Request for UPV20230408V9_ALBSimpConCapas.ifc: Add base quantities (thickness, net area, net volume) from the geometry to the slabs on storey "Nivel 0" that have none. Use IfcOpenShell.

First a look at what the model holds.

```python
import ifcopenshell
import ifcopenshell.util.element
import ifcopenshell.util.unit

model = ifcopenshell.open("UPV20230408V9_ALBSimpConCapas.ifc")
print(model.schema)
for unit_type in ("LENGTHUNIT", "AREAUNIT", "VOLUMEUNIT"):
    print(unit_type, ifcopenshell.util.unit.calculate_unit_scale(model, unit_type))
storey = next(s for s in model.by_type("IfcBuildingStorey") if s.Name == "Nivel 0")
slabs = [e for e in ifcopenshell.util.element.get_decomposition(storey) if e.is_a("IfcSlab")]
for e in sorted(slabs, key=lambda e: e.id()):
    print(e.id(), e.is_a(), e.Name, list(ifcopenshell.util.element.get_psets(e, qtos_only=True)), sep=" | ")
```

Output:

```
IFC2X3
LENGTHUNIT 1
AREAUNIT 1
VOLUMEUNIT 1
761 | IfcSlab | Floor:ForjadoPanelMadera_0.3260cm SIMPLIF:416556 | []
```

```python
import ifcopenshell
import ifcopenshell.api.pset
import ifcopenshell.geom
import ifcopenshell.util.element
import ifcopenshell.util.shape
import ifcopenshell.util.unit

model = ifcopenshell.open("UPV20230408V9_ALBSimpConCapas.ifc")
unit_scale = ifcopenshell.util.unit.calculate_unit_scale(model)
area_scale = ifcopenshell.util.unit.calculate_unit_scale(model, "AREAUNIT")
volume_scale = ifcopenshell.util.unit.calculate_unit_scale(model, "VOLUMEUNIT")
settings = ifcopenshell.geom.settings()

storey = next(s for s in model.by_type("IfcBuildingStorey") if s.Name == "Nivel 0")
slabs = [e for e in ifcopenshell.util.element.get_decomposition(storey) if e.is_a("IfcSlab")]

for e in sorted(slabs, key=lambda e: e.id()):
    if ifcopenshell.util.element.get_psets(e, qtos_only=True, should_inherit=False):
        continue
    # Geometry comes back in metres, in the element's own axes.
    shape = ifcopenshell.geom.create_shape(settings, e)
    values = {
        "Width": ifcopenshell.util.shape.get_z(shape.geometry) / unit_scale,
        "NetArea": ifcopenshell.util.shape.get_footprint_area(shape.geometry) / area_scale,
        "NetVolume": ifcopenshell.util.shape.get_volume(shape.geometry) / volume_scale,
    }
    qto = ifcopenshell.api.pset.add_qto(model, product=e, name="BaseQuantities")
    ifcopenshell.api.pset.edit_qto(model, qto=qto, properties=values)
    print(e.id(), {k: round(v, 3) for k, v in values.items()})

model.write("UPV20230408V9_ALBSimpConCapas_updated.ifc")
```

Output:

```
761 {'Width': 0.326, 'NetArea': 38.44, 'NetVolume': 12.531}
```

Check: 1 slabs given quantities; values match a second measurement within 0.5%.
